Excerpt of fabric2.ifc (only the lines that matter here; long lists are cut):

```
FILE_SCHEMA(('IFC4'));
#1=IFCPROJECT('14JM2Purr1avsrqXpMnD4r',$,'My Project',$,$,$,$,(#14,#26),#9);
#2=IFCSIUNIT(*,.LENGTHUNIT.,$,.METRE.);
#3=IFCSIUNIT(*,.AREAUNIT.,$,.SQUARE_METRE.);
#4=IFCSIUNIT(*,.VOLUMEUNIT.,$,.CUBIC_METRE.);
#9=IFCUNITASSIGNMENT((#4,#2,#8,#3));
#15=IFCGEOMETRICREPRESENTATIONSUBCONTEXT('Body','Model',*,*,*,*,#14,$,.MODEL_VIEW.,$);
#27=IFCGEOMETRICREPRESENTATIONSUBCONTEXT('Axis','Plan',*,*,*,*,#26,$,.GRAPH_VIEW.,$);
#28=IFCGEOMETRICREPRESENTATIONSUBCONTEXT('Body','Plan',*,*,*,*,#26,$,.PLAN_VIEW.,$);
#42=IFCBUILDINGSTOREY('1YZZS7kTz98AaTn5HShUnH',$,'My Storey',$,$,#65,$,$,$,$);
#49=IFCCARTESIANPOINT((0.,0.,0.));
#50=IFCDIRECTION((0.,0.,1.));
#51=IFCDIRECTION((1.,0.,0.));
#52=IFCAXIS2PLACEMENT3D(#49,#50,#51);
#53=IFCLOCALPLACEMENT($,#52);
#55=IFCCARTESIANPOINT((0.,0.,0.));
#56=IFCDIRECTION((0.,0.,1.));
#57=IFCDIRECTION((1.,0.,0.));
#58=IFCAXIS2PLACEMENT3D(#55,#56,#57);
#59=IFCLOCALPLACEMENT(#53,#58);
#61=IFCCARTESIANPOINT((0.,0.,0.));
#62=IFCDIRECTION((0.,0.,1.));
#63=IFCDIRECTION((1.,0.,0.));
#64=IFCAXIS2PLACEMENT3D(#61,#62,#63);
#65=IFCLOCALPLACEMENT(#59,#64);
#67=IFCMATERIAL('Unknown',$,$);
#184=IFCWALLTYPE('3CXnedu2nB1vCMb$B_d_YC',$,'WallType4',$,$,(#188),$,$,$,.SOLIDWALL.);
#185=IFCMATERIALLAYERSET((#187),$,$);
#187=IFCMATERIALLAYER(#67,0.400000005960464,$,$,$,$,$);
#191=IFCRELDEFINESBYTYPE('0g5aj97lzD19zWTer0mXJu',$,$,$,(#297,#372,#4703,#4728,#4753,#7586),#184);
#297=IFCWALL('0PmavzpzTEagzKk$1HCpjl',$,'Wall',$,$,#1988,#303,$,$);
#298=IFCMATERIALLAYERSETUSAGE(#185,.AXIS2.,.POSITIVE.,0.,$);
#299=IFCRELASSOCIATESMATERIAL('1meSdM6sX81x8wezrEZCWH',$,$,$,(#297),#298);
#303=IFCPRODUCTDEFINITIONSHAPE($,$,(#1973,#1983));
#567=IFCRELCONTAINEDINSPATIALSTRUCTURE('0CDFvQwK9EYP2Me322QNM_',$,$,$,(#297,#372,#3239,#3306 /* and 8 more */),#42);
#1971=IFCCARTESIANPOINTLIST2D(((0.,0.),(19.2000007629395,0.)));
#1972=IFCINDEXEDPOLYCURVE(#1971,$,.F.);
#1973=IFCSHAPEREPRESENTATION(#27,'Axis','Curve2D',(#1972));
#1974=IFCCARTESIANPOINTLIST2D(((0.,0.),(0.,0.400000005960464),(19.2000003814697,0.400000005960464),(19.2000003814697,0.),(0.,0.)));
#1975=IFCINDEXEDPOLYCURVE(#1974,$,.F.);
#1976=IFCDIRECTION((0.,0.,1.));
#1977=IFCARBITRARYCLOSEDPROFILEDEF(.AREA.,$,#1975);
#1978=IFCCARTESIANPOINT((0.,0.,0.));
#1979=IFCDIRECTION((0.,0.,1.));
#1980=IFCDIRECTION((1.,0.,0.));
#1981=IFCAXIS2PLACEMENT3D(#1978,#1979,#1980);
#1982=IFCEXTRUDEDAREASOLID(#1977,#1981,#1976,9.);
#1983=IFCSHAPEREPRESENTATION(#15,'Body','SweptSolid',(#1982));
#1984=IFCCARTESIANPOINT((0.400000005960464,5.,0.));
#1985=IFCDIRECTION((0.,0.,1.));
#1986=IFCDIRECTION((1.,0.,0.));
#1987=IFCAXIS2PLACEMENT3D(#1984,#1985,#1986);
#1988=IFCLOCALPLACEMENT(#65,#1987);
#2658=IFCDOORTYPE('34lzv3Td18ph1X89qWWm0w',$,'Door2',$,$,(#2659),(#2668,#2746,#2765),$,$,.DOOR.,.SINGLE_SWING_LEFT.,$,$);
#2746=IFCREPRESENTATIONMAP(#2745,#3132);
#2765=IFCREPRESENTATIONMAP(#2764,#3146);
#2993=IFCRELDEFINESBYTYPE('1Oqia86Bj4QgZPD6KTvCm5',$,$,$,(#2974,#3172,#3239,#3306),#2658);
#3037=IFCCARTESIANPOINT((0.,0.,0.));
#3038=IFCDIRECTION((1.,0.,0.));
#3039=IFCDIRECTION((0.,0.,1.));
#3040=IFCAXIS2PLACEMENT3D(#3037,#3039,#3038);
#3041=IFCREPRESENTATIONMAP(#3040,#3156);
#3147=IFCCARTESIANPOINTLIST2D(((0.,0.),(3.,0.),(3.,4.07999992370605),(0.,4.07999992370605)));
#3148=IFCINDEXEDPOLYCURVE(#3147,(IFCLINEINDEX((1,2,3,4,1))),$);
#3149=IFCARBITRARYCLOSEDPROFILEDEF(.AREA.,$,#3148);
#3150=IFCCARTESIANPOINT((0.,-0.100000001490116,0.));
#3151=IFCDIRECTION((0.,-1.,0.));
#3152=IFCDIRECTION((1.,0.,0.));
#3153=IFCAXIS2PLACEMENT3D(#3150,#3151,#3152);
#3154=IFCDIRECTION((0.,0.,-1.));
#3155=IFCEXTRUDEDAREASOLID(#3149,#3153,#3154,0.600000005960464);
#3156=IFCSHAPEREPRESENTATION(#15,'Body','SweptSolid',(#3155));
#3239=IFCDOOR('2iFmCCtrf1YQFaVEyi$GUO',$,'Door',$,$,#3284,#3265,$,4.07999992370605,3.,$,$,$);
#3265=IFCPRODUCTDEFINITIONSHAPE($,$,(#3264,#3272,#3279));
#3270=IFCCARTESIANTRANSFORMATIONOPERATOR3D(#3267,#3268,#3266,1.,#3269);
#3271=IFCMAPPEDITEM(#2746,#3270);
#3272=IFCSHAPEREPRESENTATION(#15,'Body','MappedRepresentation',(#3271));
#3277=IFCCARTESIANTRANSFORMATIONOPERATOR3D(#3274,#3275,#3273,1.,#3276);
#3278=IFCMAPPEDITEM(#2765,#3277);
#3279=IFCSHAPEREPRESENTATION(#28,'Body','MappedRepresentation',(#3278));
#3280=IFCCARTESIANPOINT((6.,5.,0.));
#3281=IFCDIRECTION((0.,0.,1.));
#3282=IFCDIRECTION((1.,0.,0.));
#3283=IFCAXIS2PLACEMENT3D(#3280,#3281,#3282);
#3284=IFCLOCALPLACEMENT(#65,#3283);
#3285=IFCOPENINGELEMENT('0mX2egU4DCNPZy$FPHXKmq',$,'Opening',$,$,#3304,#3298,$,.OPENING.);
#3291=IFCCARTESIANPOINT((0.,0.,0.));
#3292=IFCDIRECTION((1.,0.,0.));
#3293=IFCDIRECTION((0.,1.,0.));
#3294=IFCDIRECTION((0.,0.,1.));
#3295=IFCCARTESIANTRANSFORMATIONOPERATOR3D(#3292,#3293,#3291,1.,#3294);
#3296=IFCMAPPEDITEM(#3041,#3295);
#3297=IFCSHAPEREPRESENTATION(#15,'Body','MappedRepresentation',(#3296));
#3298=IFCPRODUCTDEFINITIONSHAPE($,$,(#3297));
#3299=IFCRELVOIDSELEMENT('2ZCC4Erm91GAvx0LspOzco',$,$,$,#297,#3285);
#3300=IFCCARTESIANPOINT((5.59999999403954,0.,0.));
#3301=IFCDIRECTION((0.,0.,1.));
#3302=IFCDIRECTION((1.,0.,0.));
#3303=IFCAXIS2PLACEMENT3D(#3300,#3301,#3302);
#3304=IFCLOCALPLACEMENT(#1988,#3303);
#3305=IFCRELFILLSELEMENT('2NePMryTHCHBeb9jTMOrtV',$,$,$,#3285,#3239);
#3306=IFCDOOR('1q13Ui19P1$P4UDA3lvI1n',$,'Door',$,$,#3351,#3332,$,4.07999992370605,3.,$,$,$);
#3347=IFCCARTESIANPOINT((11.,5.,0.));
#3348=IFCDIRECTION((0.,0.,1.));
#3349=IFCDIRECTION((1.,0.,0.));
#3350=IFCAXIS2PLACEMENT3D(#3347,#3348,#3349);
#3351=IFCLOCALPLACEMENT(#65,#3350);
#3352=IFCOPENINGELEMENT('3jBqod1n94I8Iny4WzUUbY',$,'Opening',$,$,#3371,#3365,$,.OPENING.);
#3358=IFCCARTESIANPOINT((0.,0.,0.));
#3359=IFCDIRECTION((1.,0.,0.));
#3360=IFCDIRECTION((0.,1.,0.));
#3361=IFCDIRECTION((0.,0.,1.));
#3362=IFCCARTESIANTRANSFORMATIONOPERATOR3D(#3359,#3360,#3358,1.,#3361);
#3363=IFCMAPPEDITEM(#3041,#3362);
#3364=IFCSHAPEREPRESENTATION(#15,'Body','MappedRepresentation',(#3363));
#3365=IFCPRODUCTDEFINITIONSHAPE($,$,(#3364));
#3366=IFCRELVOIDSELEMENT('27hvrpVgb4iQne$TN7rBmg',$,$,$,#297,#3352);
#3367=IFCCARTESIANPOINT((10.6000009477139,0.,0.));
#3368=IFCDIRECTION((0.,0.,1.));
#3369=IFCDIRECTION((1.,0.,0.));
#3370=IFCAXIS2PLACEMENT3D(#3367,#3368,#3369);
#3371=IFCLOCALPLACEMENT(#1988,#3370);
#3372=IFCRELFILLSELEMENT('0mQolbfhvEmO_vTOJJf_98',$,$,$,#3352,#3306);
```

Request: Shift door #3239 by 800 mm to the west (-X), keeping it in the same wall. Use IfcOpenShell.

```python
import ifcopenshell
import ifcopenshell.api.geometry
import ifcopenshell.util.placement

model = ifcopenshell.open("fabric2.ifc")

door = model.by_guid("2iFmCCtrf1YQFaVEyi$GUO")
opening = door.FillsVoids[0].RelatingOpeningElement
wall = opening.VoidsElements[0].RelatingBuildingElement

wall_matrix = ifcopenshell.util.placement.get_local_placement(wall.ObjectPlacement)
shift = wall_matrix[:3, 0] * -0.8
before = ifcopenshell.util.placement.get_local_placement(door.ObjectPlacement)[:3, 3].copy()

# The door is not placed relative to its opening, so move both.
for product in (opening, door):
    matrix = ifcopenshell.util.placement.get_local_placement(product.ObjectPlacement)
    matrix[:3, 3] += shift
    ifcopenshell.api.geometry.edit_object_placement(model, product=product, matrix=matrix, is_si=False)

after = ifcopenshell.util.placement.get_local_placement(door.ObjectPlacement)[:3, 3]
print("door moved by", (after - before).round(3) + 0.0)

model.write("fabric2_v2.ifc")
```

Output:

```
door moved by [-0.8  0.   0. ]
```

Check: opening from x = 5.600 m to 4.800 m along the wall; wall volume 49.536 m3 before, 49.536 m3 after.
